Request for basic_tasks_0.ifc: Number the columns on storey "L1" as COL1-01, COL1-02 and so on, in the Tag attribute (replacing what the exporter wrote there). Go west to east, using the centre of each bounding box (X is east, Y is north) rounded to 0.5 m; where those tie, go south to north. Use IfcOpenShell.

First a look at what the model holds.

```python
import ifcopenshell
import ifcopenshell.util.element
import ifcopenshell.util.placement

model = ifcopenshell.open("basic_tasks_0.ifc")
print(model.schema)
storey = next(s for s in model.by_type("IfcBuildingStorey") if s.Name == "L1")
columns = [e for e in ifcopenshell.util.element.get_decomposition(storey) if e.is_a("IfcColumn")]
for e in sorted(columns, key=lambda e: e.id()):
    origin = ifcopenshell.util.placement.get_local_placement(e.ObjectPlacement)[:3, 3]
    print(e.id(), e.Tag, e.Name, origin.round(2) + 0.0, sep=" | ")
```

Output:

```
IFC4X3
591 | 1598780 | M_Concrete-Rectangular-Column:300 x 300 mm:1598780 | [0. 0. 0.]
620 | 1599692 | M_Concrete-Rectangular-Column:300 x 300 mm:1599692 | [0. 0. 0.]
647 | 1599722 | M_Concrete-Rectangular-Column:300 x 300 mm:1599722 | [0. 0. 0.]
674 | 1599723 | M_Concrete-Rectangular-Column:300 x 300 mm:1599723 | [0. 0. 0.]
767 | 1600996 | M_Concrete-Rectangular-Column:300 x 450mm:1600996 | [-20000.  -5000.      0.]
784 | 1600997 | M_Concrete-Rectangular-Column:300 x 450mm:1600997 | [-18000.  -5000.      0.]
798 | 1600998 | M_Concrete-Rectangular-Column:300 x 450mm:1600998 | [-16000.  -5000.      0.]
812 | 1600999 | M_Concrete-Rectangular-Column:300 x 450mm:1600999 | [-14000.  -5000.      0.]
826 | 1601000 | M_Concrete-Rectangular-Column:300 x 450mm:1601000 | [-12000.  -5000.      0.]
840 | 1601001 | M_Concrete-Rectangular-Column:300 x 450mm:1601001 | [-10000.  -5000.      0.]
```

```python
import ifcopenshell
import ifcopenshell.geom
import ifcopenshell.util.element
import ifcopenshell.util.shape

model = ifcopenshell.open("basic_tasks_0.ifc")
settings = ifcopenshell.geom.settings()
settings.set("use-world-coords", True)


def centre(element):
    shape = ifcopenshell.geom.create_shape(settings, element)
    return ifcopenshell.util.shape.get_bbox_centroid(shape.geometry)


storey = next(s for s in model.by_type("IfcBuildingStorey") if s.Name == "L1")
columns = [e for e in ifcopenshell.util.element.get_decomposition(storey) if e.is_a("IfcColumn")]

# Insertion points can sit at a corner or the storey origin, so sort by the geometry (in metres).
centres = {e: centre(e) for e in columns}
columns.sort(key=lambda e: (round(centres[e][0] / 0.5), centres[e][1]))

for i, e in enumerate(columns, start=1):
    number = f"COL1-{i:02d}"
    e.Tag = number
    print(e.id(), number)

model.write("basic_tasks_0_edited.ifc")
```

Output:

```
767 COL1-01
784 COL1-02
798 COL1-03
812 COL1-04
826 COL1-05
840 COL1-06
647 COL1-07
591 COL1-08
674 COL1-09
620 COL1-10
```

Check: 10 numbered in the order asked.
